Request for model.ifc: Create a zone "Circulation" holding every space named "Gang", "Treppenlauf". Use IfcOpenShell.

First a look at what the model holds.

```python
import ifcopenshell

model = ifcopenshell.open("model.ifc")
print(model.schema)
seen = {}
for space in model.by_type("IfcSpace"):
    seen[space.LongName] = seen.get(space.LongName, 0) + 1
for name, count in sorted(seen.items(), key=str):
    print(count, "x", name)
print("zones:", [z.Name for z in model.by_type("IfcZone")][:20])
```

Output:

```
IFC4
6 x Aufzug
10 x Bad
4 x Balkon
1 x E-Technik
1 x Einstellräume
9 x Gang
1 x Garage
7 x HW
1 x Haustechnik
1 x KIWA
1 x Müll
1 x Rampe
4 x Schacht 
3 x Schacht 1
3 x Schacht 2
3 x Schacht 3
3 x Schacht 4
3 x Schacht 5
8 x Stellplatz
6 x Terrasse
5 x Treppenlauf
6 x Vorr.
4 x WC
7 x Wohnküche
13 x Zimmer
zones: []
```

```python
import ifcopenshell
import ifcopenshell.api.group
import ifcopenshell.api.root

model = ifcopenshell.open("model.ifc")

names = {"Gang", "Treppenlauf"}
spaces = [s for s in model.by_type("IfcSpace") if s.LongName in names]

zone = ifcopenshell.api.root.create_entity(model, ifc_class="IfcZone", name="Circulation")
ifcopenshell.api.group.assign_group(model, products=spaces, group=zone)
print(len(spaces), "spaces in", zone.Name)

model.write("model_v2.ifc")
```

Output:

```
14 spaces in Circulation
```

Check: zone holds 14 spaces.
